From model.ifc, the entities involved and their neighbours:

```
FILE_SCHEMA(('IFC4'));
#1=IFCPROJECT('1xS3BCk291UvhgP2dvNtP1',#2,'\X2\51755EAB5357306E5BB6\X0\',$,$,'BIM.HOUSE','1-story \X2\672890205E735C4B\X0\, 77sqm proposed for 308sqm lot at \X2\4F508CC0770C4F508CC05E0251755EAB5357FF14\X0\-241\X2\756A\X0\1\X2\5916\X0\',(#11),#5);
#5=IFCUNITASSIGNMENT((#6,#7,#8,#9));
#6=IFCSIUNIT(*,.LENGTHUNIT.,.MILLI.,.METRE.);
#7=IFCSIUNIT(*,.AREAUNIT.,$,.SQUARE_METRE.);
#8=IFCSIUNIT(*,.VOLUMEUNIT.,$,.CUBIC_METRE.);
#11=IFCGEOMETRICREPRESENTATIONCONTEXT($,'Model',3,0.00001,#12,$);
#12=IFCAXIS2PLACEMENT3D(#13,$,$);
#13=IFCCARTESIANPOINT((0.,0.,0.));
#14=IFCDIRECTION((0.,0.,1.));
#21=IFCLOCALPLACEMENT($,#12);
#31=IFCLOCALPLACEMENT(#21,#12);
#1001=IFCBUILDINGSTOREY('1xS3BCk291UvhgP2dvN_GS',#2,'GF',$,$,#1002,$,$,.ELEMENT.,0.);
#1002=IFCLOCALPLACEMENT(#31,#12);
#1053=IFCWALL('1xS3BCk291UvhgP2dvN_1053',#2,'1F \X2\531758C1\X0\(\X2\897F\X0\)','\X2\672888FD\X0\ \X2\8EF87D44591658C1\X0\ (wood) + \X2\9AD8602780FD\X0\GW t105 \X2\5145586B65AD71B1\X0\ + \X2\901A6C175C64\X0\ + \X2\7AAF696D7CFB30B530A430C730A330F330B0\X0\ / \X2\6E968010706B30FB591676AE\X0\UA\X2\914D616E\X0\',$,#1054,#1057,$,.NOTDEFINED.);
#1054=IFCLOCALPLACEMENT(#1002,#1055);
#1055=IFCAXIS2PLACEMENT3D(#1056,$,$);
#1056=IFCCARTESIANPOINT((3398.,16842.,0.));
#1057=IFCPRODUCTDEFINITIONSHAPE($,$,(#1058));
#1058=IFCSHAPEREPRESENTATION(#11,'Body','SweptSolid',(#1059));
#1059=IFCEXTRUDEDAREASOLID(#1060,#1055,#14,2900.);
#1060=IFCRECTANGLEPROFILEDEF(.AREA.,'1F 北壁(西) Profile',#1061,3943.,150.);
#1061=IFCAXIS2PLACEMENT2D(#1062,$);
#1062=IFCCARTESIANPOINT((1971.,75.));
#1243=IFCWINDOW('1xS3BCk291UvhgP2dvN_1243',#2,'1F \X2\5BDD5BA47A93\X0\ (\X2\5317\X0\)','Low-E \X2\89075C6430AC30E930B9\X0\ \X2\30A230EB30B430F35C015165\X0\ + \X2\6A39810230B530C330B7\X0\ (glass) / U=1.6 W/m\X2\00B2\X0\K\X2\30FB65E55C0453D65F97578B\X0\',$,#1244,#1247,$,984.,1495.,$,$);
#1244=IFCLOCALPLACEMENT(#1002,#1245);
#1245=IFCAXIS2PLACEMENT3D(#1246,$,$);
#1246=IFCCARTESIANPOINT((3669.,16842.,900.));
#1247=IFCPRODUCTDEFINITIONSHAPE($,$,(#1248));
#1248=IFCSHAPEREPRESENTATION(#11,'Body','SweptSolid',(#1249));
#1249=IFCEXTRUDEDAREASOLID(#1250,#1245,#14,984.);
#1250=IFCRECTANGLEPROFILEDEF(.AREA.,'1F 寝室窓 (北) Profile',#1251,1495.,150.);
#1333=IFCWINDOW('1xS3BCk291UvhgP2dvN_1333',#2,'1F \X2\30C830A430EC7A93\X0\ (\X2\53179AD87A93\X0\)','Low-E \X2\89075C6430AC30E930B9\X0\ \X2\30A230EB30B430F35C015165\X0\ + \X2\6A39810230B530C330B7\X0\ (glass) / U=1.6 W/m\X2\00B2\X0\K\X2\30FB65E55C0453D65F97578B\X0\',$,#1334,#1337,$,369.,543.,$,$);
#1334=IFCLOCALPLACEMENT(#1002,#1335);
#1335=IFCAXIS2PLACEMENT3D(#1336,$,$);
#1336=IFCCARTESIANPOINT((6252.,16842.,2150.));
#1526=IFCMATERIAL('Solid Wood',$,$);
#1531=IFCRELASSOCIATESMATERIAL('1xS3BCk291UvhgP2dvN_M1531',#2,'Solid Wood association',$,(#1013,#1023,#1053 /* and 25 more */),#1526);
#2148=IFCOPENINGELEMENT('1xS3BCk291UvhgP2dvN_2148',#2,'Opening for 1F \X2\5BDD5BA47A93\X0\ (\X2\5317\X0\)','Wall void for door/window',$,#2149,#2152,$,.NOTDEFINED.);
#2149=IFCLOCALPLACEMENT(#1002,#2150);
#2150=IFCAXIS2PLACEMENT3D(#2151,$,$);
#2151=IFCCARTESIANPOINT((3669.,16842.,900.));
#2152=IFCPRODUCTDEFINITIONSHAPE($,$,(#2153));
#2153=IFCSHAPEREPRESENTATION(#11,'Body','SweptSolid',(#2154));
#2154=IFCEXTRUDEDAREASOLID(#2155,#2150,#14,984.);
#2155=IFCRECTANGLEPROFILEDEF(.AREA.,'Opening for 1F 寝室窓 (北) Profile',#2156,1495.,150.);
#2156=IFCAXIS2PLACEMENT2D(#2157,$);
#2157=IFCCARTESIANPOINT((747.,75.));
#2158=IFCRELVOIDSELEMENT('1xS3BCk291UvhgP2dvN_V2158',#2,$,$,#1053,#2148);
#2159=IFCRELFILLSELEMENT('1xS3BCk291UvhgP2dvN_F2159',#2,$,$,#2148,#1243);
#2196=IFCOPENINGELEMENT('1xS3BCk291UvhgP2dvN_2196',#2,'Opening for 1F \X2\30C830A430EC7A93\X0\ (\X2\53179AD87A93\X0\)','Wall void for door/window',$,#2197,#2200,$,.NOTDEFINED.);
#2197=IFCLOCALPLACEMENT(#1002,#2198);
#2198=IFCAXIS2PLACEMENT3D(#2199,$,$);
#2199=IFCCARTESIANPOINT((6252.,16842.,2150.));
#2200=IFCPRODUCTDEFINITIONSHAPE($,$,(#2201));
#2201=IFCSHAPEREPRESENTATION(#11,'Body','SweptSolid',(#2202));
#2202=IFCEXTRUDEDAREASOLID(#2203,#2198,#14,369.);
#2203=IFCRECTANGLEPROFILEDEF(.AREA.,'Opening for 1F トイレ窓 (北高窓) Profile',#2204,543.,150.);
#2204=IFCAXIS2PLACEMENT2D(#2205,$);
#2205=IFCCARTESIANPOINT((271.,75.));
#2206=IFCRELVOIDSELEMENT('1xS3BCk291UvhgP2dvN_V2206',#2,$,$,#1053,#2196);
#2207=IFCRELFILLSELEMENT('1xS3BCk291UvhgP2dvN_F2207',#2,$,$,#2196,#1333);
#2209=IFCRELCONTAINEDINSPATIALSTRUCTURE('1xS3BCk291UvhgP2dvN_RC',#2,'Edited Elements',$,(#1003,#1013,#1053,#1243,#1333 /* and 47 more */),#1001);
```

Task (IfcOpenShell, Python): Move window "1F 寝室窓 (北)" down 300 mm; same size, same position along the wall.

```python
import numpy as np
import ifcopenshell
import ifcopenshell.api.geometry
import ifcopenshell.util.placement
import ifcopenshell.util.unit

model = ifcopenshell.open("model.ifc")
unit_scale = ifcopenshell.util.unit.calculate_unit_scale(model)

window = model.by_guid("1xS3BCk291UvhgP2dvN_1243")
opening = window.FillsVoids[0].RelatingOpeningElement
dz = -300.0

shift = np.array([0.0, 0.0, dz])
# The window is not placed relative to its opening, so move both.
for product in (opening, window):
    matrix = ifcopenshell.util.placement.get_local_placement(product.ObjectPlacement)
    matrix[:3, 3] += shift
    ifcopenshell.api.geometry.edit_object_placement(model, product=product, matrix=matrix, is_si=False)

print(f"moved by {dz * unit_scale:+.3f} m")

model.write("model_rev.ifc")
```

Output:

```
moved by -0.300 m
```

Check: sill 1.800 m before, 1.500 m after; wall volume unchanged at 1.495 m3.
